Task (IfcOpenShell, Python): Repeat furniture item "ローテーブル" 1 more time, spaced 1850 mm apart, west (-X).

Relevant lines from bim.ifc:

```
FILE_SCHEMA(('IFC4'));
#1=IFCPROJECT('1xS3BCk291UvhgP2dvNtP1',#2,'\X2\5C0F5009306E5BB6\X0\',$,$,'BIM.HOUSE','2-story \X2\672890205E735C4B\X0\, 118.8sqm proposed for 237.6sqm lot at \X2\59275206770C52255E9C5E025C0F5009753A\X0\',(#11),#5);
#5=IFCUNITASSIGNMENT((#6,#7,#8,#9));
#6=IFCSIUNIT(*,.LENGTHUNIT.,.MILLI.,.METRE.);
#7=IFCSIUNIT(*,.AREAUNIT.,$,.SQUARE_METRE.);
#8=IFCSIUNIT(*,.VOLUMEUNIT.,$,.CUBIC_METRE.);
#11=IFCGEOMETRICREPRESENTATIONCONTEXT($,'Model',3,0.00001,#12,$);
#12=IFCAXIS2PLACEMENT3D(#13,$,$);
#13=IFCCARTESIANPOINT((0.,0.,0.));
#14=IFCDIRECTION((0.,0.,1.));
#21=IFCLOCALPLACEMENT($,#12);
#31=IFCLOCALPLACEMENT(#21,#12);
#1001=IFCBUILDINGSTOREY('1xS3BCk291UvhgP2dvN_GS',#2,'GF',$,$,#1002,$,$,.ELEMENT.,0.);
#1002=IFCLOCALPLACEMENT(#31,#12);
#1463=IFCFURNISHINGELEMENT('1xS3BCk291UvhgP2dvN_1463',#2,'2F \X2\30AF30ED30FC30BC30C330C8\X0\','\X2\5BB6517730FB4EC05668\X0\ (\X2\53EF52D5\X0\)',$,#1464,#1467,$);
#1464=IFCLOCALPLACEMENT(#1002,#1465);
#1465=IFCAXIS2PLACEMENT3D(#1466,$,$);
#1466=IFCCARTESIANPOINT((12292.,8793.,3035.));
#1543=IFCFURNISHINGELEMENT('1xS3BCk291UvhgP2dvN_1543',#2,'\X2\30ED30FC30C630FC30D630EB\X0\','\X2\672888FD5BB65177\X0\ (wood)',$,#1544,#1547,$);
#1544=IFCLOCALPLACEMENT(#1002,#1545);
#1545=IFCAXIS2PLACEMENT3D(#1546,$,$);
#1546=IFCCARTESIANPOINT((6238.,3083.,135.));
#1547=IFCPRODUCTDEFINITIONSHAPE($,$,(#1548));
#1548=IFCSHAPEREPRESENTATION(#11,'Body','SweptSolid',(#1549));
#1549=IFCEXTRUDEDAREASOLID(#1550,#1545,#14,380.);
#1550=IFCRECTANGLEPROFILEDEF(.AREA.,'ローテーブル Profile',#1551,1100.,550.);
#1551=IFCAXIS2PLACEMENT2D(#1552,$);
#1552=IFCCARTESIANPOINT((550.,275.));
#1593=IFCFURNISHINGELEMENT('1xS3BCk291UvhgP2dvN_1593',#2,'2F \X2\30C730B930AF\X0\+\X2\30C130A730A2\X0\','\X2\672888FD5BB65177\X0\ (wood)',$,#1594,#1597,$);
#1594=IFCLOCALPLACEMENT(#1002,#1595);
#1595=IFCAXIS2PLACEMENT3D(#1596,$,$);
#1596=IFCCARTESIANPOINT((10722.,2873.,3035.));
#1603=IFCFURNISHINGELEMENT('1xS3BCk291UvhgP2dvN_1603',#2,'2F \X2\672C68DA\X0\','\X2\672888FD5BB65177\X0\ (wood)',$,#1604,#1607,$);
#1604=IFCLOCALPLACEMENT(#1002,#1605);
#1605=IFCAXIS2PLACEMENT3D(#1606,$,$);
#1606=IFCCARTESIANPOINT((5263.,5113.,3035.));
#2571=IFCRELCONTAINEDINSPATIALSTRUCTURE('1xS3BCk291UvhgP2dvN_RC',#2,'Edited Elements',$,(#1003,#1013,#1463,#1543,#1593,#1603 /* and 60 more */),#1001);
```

```python
import numpy as np
import ifcopenshell
import ifcopenshell.api.geometry
import ifcopenshell.api.root
import ifcopenshell.util.element
import ifcopenshell.util.placement
import ifcopenshell.util.unit

model = ifcopenshell.open("bim.ifc")
unit_scale = ifcopenshell.util.unit.calculate_unit_scale(model)


def reuse_history(source, copy):
    """copy_class also copies each property set's owner history, people and application; keep the originals."""
    for rel in copy.IsDefinedBy:
        if rel.is_a("IfcRelDefinesByProperties") and (history := rel.RelatingPropertyDefinition.OwnerHistory):
            rel.RelatingPropertyDefinition.OwnerHistory = source.OwnerHistory
            ifcopenshell.util.element.remove_deep2(model, history)


source = model.by_id(1543)
base = ifcopenshell.util.placement.get_local_placement(source.ObjectPlacement)
step = np.array([-1.0, 0.0, 0.0]) * 1.85 / unit_scale

for i in range(1, 2):
    copy = ifcopenshell.api.root.copy_class(model, product=source)
    copy.Representation = ifcopenshell.util.element.copy_deep(
        model, source.Representation, exclude=["IfcGeometricRepresentationContext", "IfcRepresentationMap"]
    )
    reuse_history(source, copy)
    matrix = base.copy()
    matrix[:3, 3] += i * step
    print("added at", matrix[:3, 3].round(3) + 0.0)
    ifcopenshell.api.geometry.edit_object_placement(model, product=copy, matrix=matrix, is_si=False)

model.write("bim-out.ifc")
```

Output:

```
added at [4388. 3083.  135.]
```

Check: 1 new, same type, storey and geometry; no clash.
